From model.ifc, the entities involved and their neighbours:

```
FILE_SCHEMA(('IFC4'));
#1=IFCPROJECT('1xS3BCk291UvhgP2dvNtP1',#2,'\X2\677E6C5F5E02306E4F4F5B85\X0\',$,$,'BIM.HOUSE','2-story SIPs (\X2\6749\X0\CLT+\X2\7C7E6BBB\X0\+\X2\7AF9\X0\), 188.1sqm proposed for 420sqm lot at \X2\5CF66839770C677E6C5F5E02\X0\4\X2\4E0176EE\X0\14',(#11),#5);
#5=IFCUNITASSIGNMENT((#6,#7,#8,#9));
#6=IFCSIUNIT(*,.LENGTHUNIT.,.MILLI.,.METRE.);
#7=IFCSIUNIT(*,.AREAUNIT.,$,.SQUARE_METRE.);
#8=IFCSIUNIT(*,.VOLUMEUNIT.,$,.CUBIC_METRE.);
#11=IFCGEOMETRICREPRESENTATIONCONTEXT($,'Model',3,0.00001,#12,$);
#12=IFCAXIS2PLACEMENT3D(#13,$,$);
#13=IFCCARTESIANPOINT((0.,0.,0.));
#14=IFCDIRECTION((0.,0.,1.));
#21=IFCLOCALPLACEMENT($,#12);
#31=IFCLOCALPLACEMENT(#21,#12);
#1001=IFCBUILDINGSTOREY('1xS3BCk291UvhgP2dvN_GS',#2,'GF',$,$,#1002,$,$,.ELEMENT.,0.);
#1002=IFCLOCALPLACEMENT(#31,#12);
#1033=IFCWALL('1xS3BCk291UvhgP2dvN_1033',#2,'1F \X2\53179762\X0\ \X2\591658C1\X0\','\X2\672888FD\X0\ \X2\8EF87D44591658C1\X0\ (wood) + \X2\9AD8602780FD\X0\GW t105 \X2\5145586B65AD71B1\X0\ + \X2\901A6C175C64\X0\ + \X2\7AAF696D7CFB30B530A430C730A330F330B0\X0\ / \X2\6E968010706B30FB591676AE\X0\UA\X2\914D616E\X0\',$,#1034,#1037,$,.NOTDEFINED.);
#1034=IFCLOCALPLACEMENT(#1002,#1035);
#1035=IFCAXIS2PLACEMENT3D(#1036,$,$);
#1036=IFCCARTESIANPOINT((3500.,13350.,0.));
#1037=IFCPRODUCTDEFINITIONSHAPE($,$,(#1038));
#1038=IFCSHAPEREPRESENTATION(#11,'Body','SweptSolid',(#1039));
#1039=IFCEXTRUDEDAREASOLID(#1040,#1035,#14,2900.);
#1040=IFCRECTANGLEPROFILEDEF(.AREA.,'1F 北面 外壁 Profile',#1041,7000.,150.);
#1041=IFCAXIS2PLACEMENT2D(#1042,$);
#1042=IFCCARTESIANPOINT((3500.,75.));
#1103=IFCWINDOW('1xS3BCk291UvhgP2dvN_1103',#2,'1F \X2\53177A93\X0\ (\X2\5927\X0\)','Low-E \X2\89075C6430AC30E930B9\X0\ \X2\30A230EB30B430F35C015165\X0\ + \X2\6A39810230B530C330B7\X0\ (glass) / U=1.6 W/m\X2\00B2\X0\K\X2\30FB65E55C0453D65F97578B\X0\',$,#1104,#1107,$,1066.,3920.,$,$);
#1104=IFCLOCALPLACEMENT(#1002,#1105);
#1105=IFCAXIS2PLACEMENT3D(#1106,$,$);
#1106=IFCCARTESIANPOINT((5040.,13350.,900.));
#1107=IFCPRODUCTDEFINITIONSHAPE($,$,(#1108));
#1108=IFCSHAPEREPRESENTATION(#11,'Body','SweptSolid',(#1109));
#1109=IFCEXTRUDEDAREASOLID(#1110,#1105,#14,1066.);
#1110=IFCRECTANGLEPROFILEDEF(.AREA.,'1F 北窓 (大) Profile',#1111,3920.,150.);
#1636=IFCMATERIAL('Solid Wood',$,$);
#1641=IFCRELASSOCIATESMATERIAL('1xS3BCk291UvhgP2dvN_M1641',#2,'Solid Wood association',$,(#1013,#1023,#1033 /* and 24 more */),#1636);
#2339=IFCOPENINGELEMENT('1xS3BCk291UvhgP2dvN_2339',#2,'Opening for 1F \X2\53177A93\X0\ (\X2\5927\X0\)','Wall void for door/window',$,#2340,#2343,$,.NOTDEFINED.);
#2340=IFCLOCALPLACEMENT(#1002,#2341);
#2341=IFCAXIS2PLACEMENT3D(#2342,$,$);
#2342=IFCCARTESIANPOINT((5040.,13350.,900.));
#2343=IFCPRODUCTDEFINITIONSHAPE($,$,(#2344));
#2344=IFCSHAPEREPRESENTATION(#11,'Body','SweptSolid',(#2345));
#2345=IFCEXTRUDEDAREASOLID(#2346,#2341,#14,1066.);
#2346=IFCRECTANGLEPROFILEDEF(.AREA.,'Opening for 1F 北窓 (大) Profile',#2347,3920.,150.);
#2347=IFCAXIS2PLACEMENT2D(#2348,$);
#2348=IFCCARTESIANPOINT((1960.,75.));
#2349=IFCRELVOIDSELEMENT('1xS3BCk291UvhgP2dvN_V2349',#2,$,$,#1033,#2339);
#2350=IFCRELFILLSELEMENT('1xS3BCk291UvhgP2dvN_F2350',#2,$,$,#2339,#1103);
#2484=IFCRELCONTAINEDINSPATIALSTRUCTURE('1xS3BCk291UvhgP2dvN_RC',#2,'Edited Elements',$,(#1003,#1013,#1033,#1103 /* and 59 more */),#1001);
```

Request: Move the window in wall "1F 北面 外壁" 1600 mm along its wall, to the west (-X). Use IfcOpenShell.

```python
import ifcopenshell
import ifcopenshell.api.geometry
import ifcopenshell.util.placement

model = ifcopenshell.open("model.ifc")

window = model.by_guid("1xS3BCk291UvhgP2dvN_1103")
opening = window.FillsVoids[0].RelatingOpeningElement
wall = opening.VoidsElements[0].RelatingBuildingElement

wall_matrix = ifcopenshell.util.placement.get_local_placement(wall.ObjectPlacement)
shift = wall_matrix[:3, 0] * -1600.0
before = ifcopenshell.util.placement.get_local_placement(window.ObjectPlacement)[:3, 3].copy()

# The window is not placed relative to its opening, so move both.
for product in (opening, window):
    matrix = ifcopenshell.util.placement.get_local_placement(product.ObjectPlacement)
    matrix[:3, 3] += shift
    ifcopenshell.api.geometry.edit_object_placement(model, product=product, matrix=matrix, is_si=False)

after = ifcopenshell.util.placement.get_local_placement(window.ObjectPlacement)[:3, 3]
print("window moved by", (after - before).round(3) + 0.0)

model.write("model_rev.ifc")
```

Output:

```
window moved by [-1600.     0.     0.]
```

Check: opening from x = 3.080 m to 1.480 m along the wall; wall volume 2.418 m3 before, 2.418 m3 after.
